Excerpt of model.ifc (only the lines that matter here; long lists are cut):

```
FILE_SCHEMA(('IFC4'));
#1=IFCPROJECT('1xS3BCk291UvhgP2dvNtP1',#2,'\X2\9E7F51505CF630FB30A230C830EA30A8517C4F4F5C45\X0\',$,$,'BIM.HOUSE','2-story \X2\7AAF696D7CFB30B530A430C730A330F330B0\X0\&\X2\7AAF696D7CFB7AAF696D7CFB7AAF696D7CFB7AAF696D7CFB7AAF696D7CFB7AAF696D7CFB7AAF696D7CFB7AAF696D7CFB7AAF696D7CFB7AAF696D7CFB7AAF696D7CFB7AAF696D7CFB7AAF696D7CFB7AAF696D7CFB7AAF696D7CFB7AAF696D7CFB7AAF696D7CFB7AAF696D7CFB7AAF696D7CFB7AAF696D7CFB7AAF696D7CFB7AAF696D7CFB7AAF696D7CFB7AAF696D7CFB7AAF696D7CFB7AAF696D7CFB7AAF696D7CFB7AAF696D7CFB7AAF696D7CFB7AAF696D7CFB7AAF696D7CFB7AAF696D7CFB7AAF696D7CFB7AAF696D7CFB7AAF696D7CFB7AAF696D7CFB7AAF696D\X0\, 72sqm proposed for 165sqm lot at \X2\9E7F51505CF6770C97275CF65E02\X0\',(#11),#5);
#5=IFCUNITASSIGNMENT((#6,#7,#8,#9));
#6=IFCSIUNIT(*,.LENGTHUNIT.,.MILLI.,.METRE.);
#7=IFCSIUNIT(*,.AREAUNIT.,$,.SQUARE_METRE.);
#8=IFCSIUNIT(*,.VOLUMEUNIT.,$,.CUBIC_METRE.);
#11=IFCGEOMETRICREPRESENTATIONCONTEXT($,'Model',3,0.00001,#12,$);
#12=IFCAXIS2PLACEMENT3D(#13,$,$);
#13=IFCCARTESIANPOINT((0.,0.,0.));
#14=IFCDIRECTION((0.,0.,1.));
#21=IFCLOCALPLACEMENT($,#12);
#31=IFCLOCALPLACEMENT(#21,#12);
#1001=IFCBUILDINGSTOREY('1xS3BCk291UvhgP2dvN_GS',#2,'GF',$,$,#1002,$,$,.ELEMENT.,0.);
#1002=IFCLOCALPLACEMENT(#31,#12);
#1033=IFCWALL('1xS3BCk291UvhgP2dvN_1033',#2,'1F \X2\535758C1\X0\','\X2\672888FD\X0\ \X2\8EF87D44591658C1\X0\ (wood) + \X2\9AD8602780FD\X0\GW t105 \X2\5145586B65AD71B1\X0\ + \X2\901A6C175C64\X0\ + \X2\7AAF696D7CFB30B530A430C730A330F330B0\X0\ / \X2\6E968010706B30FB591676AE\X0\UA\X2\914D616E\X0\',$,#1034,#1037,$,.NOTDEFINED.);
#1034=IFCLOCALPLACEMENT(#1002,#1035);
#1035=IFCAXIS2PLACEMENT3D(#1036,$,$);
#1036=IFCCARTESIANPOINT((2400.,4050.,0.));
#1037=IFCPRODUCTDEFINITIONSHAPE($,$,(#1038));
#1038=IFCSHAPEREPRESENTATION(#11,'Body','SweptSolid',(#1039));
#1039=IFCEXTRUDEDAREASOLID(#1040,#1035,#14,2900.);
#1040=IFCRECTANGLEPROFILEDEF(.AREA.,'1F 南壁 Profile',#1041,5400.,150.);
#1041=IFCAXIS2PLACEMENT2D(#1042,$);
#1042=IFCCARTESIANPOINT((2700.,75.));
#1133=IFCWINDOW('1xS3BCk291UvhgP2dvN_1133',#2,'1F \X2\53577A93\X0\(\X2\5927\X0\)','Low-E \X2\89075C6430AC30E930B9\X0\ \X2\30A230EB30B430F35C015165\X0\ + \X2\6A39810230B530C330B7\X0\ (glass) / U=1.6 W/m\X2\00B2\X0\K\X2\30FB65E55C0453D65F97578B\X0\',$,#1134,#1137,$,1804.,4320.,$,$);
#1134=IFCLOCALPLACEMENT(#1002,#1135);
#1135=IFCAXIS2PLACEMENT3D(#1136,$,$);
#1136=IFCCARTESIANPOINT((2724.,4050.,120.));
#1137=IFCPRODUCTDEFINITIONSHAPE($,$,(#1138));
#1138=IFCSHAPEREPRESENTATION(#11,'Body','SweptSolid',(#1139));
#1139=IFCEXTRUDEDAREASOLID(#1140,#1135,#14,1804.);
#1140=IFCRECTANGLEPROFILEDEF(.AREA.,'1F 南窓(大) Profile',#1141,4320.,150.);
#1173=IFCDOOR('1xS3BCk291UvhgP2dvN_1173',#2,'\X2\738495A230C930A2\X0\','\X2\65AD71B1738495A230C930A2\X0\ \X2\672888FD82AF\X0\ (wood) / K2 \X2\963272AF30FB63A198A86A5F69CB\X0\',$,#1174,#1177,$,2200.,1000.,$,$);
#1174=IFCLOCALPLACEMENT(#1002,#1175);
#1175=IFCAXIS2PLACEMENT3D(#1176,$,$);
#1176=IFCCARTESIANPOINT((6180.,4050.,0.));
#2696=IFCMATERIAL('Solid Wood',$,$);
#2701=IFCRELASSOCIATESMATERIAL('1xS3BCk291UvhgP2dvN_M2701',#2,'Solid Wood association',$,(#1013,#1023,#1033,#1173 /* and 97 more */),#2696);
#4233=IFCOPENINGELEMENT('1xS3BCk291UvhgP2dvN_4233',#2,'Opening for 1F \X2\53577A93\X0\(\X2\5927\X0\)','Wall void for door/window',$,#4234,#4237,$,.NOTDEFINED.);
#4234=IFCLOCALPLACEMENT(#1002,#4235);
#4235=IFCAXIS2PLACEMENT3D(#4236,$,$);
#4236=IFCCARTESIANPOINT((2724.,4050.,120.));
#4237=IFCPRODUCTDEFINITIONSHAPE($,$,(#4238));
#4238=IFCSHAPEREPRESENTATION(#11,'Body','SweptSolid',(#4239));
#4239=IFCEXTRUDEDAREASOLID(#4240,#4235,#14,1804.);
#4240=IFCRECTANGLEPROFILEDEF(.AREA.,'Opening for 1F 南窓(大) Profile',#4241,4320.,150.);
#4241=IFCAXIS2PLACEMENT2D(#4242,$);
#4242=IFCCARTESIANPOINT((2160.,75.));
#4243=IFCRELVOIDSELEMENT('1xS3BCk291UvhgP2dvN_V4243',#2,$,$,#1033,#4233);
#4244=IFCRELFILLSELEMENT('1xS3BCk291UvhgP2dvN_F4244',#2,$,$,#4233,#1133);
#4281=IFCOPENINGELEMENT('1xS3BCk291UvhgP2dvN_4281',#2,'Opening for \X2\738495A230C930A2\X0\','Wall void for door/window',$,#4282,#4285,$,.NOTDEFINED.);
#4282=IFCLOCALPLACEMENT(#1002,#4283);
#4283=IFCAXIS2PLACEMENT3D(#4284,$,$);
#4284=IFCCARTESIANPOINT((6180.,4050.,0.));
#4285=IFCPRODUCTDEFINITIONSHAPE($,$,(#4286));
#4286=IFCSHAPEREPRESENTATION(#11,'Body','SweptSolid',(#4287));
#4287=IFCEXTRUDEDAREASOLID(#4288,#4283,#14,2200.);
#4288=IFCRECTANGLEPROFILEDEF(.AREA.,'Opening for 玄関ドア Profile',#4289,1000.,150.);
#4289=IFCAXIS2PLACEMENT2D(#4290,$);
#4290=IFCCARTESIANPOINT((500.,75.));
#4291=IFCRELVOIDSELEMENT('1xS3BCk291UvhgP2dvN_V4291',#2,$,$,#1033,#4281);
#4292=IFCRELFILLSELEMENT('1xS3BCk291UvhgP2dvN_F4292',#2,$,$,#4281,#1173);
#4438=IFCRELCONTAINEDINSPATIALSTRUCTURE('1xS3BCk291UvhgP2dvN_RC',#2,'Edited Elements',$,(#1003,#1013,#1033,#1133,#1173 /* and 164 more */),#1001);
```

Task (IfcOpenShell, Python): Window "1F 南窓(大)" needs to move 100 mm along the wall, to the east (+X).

```python
import ifcopenshell
import ifcopenshell.api.geometry
import ifcopenshell.util.placement
import ifcopenshell.util.unit

model = ifcopenshell.open("model.ifc")
unit_scale = ifcopenshell.util.unit.calculate_unit_scale(model)

window = model.by_guid("1xS3BCk291UvhgP2dvN_1133")
opening = window.FillsVoids[0].RelatingOpeningElement
wall = opening.VoidsElements[0].RelatingBuildingElement

wall_matrix = ifcopenshell.util.placement.get_local_placement(wall.ObjectPlacement)
shift = wall_matrix[:3, 0] * 0.1 / unit_scale
before = ifcopenshell.util.placement.get_local_placement(window.ObjectPlacement)[:3, 3].copy()

# The window is not placed relative to its opening, so move both.
for product in (opening, window):
    matrix = ifcopenshell.util.placement.get_local_placement(product.ObjectPlacement)
    matrix[:3, 3] += shift
    ifcopenshell.api.geometry.edit_object_placement(model, product=product, matrix=matrix, is_si=False)

after = ifcopenshell.util.placement.get_local_placement(window.ObjectPlacement)[:3, 3]
print("window moved by", (after - before).round(3) + 0.0)

model.write("model_rev.ifc")
```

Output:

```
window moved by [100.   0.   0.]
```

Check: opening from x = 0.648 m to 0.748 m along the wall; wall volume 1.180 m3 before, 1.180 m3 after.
